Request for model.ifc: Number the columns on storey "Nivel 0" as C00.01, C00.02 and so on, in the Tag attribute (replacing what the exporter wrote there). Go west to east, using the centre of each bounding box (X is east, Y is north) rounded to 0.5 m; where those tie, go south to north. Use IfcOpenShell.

First a look at what the model holds.

```python
import ifcopenshell
import ifcopenshell.util.element
import ifcopenshell.util.placement

model = ifcopenshell.open("model.ifc")
print(model.schema)
storey = next(s for s in model.by_type("IfcBuildingStorey") if s.Name == "Nivel 0")
columns = [e for e in ifcopenshell.util.element.get_decomposition(storey) if e.is_a("IfcColumn")]
for e in sorted(columns, key=lambda e: e.id()):
    origin = ifcopenshell.util.placement.get_local_placement(e.ObjectPlacement)[:3, 3]
    print(e.id(), e.Tag, e.Name, origin.round(2) + 0.0, sep=" | ")
```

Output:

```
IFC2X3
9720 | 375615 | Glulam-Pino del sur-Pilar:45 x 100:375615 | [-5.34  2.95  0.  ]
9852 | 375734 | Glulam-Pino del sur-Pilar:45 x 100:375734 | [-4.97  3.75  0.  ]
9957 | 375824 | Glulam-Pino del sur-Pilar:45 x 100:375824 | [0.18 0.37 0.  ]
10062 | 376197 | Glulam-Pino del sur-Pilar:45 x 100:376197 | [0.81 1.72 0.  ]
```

```python
import ifcopenshell
import ifcopenshell.geom
import ifcopenshell.util.element
import ifcopenshell.util.shape

model = ifcopenshell.open("model.ifc")
settings = ifcopenshell.geom.settings()
settings.set("use-world-coords", True)


def centre(element):
    shape = ifcopenshell.geom.create_shape(settings, element)
    return ifcopenshell.util.shape.get_bbox_centroid(shape.geometry)


storey = next(s for s in model.by_type("IfcBuildingStorey") if s.Name == "Nivel 0")
columns = [e for e in ifcopenshell.util.element.get_decomposition(storey) if e.is_a("IfcColumn")]

# Insertion points can sit at a corner or the storey origin, so sort by the geometry (in metres).
centres = {e: centre(e) for e in columns}
columns.sort(key=lambda e: (round(centres[e][0] / 0.5), centres[e][1]))

for i, e in enumerate(columns, start=1):
    number = f"C00.{i:02d}"
    e.Tag = number
    print(e.id(), number)

model.write("model_updated.ifc")
```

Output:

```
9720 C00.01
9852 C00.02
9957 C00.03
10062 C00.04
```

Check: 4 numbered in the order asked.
